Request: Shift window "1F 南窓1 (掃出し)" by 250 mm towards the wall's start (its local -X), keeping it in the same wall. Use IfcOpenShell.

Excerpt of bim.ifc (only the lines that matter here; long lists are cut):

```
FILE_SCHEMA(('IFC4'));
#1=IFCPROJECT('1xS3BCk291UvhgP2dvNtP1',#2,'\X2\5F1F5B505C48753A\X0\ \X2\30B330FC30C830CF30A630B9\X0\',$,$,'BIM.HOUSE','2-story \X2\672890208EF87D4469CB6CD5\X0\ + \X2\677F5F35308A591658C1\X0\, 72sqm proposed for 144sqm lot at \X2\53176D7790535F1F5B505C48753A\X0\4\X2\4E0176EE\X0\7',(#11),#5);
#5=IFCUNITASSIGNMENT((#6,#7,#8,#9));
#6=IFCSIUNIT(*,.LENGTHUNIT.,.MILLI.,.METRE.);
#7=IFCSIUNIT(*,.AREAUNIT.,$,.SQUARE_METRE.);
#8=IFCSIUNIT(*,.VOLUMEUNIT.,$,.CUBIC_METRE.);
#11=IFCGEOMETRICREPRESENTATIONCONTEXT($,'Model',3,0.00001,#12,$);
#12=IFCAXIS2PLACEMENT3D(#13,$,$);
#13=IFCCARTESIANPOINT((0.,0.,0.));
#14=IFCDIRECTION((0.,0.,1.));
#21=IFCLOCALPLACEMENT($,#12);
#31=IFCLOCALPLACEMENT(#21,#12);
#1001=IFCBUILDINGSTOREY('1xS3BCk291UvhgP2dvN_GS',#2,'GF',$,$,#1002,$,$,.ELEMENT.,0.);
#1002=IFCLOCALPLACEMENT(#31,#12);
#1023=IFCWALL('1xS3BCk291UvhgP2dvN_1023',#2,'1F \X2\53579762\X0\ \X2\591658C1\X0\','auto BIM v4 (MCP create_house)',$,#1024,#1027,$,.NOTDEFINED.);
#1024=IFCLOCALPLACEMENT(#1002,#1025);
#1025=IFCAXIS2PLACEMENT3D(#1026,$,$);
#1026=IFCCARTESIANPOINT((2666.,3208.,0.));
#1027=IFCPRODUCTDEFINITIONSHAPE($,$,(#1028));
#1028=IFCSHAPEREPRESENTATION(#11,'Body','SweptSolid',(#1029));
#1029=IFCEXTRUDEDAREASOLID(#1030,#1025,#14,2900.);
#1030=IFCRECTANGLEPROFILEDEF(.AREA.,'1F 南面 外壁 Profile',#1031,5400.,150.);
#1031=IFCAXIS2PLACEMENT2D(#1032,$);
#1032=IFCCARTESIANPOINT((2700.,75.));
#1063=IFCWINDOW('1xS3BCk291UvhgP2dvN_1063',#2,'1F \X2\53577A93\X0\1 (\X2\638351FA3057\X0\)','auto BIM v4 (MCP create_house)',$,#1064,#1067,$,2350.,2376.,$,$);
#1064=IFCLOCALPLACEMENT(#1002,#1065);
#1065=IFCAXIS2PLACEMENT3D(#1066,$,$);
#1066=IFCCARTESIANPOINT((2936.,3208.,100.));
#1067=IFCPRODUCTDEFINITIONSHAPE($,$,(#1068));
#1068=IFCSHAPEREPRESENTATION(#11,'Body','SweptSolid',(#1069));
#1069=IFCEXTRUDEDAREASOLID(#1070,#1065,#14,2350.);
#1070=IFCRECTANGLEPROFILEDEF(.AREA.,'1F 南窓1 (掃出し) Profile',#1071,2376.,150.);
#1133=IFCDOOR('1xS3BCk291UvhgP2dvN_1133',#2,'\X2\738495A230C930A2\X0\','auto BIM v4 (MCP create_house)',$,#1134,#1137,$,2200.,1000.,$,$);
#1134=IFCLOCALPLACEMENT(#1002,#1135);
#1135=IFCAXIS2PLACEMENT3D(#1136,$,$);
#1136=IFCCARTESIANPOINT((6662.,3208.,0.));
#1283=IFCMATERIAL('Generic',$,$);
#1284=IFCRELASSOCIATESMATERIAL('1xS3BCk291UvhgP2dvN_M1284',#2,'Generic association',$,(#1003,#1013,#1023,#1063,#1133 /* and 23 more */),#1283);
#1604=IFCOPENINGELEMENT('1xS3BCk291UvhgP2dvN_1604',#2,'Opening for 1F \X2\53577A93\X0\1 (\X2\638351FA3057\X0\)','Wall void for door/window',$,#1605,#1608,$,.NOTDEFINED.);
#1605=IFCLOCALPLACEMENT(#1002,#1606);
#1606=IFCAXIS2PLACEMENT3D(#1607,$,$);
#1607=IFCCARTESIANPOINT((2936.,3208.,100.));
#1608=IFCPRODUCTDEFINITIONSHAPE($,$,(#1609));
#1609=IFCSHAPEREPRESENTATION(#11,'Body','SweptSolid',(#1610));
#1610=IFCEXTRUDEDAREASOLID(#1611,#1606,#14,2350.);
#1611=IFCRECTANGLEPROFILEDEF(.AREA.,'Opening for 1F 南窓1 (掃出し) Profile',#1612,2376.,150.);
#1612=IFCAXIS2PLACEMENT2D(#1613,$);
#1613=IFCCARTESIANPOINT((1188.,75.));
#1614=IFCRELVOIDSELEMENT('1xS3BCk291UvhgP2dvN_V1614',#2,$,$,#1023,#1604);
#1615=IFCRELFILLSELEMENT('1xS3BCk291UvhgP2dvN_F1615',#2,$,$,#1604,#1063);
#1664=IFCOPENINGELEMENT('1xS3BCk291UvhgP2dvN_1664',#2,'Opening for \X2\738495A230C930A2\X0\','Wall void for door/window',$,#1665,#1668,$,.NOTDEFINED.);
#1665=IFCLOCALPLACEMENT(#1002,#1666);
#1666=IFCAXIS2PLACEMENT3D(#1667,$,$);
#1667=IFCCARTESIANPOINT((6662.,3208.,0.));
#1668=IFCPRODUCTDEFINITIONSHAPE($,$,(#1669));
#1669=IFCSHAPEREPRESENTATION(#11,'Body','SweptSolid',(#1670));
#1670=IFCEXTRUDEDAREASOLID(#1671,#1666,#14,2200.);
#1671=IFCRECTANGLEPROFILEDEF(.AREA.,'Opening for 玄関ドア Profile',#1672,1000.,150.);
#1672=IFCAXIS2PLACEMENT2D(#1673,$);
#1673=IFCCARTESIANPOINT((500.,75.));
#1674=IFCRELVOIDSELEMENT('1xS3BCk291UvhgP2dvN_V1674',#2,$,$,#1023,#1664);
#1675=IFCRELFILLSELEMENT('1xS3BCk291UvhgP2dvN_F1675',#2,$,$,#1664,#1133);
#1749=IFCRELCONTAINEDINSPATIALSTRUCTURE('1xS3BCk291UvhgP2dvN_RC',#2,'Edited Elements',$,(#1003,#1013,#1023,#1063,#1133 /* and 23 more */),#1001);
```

```python
import ifcopenshell
import ifcopenshell.api.geometry
import ifcopenshell.util.placement
import ifcopenshell.util.unit

model = ifcopenshell.open("bim.ifc")
unit_scale = ifcopenshell.util.unit.calculate_unit_scale(model)

window = model.by_guid("1xS3BCk291UvhgP2dvN_1063")
opening = window.FillsVoids[0].RelatingOpeningElement
wall = opening.VoidsElements[0].RelatingBuildingElement

wall_matrix = ifcopenshell.util.placement.get_local_placement(wall.ObjectPlacement)
shift = wall_matrix[:3, 0] * -0.25 / unit_scale
before = ifcopenshell.util.placement.get_local_placement(window.ObjectPlacement)[:3, 3].copy()

# The window is not placed relative to its opening, so move both.
for product in (opening, window):
    matrix = ifcopenshell.util.placement.get_local_placement(product.ObjectPlacement)
    matrix[:3, 3] += shift
    ifcopenshell.api.geometry.edit_object_placement(model, product=product, matrix=matrix, is_si=False)

after = ifcopenshell.util.placement.get_local_placement(window.ObjectPlacement)[:3, 3]
print("window moved by", (after - before).round(3) + 0.0)

model.write("bim_updated.ifc")
```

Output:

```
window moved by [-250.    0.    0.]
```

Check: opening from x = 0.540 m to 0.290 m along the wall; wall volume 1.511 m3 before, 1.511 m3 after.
